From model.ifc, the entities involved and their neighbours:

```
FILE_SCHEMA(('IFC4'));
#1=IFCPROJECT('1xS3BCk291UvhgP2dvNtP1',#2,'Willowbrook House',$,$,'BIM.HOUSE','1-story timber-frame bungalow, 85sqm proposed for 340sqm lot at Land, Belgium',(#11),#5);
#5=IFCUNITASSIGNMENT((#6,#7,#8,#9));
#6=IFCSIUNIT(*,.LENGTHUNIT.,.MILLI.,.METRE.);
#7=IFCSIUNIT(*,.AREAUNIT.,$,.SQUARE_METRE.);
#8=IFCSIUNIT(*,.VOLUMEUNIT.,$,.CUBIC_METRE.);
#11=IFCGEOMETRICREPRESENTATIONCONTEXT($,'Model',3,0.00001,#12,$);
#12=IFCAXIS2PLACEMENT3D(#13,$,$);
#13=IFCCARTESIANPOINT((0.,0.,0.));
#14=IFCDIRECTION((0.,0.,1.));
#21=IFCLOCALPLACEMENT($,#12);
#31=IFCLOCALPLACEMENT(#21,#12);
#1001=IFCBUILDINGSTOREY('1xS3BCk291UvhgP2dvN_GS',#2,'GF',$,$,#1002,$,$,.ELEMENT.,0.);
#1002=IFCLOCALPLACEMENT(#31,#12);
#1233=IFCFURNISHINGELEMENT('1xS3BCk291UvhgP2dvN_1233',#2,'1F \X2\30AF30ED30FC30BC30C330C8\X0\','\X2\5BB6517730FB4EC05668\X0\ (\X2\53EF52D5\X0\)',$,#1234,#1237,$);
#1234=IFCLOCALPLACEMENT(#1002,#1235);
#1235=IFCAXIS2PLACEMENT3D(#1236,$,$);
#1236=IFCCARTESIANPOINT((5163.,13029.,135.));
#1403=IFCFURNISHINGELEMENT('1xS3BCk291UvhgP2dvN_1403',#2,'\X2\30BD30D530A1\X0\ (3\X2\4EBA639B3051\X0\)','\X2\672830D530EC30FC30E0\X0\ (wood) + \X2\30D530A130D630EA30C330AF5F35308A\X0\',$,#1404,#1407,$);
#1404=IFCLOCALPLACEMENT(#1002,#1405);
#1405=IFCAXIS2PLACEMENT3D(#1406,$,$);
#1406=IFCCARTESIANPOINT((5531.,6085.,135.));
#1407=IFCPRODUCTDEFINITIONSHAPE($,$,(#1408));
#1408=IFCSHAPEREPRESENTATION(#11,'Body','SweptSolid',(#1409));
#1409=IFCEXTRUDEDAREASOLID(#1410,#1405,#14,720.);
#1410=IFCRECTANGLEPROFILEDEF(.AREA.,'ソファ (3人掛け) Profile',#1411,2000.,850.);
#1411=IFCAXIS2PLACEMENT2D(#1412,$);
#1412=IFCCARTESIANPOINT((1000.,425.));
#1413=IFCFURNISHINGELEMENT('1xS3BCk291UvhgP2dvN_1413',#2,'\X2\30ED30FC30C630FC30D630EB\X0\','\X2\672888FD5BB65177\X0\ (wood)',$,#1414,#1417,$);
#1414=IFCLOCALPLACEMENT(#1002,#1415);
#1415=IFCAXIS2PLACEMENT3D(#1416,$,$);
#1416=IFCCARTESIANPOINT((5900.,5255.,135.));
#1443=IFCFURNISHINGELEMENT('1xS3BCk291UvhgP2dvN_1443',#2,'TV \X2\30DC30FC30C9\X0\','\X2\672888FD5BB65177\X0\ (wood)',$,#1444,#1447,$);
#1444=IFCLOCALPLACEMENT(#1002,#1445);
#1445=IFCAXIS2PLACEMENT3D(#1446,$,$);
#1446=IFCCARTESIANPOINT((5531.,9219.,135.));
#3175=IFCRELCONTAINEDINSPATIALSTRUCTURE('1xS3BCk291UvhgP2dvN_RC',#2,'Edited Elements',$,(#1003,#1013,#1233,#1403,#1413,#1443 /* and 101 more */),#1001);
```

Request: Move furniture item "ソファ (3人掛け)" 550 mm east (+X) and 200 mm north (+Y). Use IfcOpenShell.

```python
import ifcopenshell
import ifcopenshell.api.geometry
import ifcopenshell.util.placement
import ifcopenshell.util.unit

model = ifcopenshell.open("model.ifc")
unit_scale = ifcopenshell.util.unit.calculate_unit_scale(model)

item = model.by_guid("1xS3BCk291UvhgP2dvN_1403")
matrix = ifcopenshell.util.placement.get_local_placement(item.ObjectPlacement)
matrix[0, 3] += 0.55 / unit_scale
matrix[1, 3] += 0.2 / unit_scale
ifcopenshell.api.geometry.edit_object_placement(model, product=item, matrix=matrix, is_si=False)

print(ifcopenshell.util.placement.get_local_placement(item.ObjectPlacement).round(3) + 0.0)

model.write("model_v2.ifc")
```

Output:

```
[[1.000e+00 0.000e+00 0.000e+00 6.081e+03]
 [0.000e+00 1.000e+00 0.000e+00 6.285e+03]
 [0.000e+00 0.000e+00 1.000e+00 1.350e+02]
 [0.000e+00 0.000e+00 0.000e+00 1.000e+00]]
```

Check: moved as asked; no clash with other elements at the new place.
